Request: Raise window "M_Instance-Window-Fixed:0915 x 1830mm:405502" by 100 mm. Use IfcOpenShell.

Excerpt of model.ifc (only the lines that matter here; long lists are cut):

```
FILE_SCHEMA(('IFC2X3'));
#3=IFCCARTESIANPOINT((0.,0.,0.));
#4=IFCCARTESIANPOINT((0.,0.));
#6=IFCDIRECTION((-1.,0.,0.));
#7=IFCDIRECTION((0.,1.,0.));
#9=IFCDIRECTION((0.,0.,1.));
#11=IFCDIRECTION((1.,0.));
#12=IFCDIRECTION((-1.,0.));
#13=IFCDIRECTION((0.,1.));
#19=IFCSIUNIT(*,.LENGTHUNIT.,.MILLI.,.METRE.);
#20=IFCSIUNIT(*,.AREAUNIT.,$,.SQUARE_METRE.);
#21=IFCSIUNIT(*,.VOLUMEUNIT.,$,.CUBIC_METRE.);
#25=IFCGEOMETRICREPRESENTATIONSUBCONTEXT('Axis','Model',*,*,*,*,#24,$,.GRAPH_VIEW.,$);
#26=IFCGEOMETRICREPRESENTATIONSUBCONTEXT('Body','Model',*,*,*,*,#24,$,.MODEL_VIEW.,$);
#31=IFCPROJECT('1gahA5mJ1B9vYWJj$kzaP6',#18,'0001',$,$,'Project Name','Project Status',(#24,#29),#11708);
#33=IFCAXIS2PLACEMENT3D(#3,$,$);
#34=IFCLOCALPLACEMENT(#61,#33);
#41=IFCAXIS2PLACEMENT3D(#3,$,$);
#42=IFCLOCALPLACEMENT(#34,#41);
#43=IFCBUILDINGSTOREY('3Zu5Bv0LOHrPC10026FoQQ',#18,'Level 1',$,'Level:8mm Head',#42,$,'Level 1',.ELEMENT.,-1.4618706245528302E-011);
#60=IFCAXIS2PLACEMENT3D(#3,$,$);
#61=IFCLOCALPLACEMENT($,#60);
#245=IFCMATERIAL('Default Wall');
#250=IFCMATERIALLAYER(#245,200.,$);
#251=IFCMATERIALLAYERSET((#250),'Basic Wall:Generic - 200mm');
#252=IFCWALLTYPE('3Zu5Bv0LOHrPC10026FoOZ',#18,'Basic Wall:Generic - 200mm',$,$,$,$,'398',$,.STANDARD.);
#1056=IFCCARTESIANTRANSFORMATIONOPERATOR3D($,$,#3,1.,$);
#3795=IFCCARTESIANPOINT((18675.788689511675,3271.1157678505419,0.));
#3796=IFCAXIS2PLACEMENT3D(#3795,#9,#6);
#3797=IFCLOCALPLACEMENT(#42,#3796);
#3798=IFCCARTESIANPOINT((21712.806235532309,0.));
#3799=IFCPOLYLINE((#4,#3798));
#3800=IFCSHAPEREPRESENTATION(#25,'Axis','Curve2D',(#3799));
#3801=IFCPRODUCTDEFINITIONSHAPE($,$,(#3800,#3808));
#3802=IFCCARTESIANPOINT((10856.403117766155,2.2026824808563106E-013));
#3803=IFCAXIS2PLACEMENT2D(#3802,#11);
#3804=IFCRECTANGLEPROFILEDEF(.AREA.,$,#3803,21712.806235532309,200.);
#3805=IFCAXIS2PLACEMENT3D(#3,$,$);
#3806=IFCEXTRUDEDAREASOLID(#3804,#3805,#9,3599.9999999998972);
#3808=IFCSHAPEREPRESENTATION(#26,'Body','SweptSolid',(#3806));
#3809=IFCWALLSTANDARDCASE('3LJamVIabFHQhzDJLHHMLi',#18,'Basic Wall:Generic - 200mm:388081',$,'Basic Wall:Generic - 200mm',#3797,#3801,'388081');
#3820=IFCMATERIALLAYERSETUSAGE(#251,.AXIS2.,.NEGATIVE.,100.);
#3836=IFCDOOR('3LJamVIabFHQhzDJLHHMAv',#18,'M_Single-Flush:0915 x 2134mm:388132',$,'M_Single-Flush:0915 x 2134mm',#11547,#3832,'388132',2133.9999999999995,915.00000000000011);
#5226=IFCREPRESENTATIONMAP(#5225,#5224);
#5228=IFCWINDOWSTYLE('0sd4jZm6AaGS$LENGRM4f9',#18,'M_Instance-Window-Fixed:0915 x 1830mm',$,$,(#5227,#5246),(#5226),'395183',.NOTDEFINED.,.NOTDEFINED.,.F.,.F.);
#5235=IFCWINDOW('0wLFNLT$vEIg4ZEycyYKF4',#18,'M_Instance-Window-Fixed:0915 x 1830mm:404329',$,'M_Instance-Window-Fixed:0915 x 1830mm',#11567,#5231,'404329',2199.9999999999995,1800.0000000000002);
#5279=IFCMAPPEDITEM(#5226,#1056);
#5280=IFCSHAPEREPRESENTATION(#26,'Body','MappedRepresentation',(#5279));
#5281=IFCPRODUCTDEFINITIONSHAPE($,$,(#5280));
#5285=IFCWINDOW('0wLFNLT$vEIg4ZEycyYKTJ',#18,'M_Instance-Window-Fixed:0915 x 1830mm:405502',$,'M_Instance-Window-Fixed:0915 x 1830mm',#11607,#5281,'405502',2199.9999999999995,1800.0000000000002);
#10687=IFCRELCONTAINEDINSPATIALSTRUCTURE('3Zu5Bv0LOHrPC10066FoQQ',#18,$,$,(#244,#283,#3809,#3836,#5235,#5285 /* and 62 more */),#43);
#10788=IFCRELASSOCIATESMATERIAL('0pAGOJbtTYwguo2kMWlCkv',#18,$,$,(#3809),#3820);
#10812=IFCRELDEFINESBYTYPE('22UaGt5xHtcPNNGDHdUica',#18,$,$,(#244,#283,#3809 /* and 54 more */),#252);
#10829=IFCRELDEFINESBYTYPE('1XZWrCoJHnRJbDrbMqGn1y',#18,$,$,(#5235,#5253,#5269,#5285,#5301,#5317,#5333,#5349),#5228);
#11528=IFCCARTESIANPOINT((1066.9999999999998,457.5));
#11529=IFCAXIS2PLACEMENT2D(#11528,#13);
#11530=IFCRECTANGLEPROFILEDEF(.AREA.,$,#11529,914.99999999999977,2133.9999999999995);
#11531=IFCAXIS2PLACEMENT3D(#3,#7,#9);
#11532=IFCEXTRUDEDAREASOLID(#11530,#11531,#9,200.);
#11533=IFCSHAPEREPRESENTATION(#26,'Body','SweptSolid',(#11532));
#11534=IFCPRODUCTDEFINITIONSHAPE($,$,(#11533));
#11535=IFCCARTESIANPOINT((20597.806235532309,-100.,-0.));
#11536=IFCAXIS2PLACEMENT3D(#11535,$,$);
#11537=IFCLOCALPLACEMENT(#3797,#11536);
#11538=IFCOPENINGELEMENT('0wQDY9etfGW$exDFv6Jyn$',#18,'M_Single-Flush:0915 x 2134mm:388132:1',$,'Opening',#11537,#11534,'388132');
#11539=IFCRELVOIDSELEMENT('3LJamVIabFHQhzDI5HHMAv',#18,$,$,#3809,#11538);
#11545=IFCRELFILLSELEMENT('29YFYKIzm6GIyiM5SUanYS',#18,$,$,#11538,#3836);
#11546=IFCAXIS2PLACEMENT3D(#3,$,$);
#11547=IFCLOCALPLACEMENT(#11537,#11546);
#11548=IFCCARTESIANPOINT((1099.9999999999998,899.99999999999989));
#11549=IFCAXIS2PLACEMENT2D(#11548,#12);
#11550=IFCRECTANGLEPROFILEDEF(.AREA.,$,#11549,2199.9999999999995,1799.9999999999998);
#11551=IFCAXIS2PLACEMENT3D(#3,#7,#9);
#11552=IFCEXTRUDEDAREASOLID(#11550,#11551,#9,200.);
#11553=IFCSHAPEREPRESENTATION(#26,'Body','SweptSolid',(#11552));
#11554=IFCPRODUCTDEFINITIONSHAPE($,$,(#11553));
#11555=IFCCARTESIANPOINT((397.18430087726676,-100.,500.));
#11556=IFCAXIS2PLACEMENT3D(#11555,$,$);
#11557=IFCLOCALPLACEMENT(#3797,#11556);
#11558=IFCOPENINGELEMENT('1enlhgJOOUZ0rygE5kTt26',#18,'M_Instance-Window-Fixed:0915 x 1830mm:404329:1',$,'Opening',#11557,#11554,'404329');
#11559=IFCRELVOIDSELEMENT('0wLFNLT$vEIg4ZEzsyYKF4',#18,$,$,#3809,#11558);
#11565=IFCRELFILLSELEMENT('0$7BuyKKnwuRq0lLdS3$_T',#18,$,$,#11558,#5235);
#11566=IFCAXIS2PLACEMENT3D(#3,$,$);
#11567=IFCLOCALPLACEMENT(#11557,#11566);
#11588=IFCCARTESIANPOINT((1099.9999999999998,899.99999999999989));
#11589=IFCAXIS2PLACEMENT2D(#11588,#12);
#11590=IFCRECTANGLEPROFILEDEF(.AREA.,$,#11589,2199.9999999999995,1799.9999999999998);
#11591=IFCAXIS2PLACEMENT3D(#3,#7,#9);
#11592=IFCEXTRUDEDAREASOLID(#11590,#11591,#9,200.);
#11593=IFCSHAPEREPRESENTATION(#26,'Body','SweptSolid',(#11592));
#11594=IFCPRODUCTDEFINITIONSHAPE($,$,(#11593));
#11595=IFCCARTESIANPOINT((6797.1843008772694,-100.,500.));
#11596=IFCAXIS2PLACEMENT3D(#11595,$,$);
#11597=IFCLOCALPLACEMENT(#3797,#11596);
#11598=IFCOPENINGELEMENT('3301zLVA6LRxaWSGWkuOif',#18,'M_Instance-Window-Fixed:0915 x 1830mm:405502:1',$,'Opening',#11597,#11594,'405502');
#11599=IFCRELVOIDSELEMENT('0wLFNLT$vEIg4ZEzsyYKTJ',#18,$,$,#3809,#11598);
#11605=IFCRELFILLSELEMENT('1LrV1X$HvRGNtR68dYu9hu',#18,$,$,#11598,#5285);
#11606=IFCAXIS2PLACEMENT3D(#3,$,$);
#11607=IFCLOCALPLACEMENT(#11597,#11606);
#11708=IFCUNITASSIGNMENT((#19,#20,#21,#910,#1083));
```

```python
import numpy as np
import ifcopenshell
import ifcopenshell.api.geometry
import ifcopenshell.util.placement
import ifcopenshell.util.unit

model = ifcopenshell.open("model.ifc")
unit_scale = ifcopenshell.util.unit.calculate_unit_scale(model)

window = model.by_guid("0wLFNLT$vEIg4ZEycyYKTJ")
opening = window.FillsVoids[0].RelatingOpeningElement
dz = 100.0

shift = np.array([0.0, 0.0, dz])
# The window is placed relative to its opening, so it follows when the opening moves.
matrix = ifcopenshell.util.placement.get_local_placement(opening.ObjectPlacement)
matrix[:3, 3] += shift
ifcopenshell.api.geometry.edit_object_placement(
    model, product=opening, matrix=matrix, is_si=False, should_transform_children=True
)

print(f"moved by {dz * unit_scale:+.3f} m")

model.write("model_v2.ifc")
```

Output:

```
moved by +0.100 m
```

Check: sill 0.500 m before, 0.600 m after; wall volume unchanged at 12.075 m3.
